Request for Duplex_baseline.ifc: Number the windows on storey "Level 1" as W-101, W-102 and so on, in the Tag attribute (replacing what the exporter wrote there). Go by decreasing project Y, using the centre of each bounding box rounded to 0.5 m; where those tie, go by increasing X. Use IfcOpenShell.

First a look at what the model holds.

```python
import ifcopenshell
import ifcopenshell.util.element
import ifcopenshell.util.placement

model = ifcopenshell.open("Duplex_baseline.ifc")
print(model.schema)
storey = next(s for s in model.by_type("IfcBuildingStorey") if s.Name == "Level 1")
windows = [e for e in ifcopenshell.util.element.get_decomposition(storey) if e.is_a("IfcWindow")]
for e in sorted(windows, key=lambda e: e.id()):
    origin = ifcopenshell.util.placement.get_local_placement(e.ObjectPlacement)[:3, 3]
    print(e.id(), e.Tag, e.Name, origin.round(2) + 0.0, sep=" | ")
```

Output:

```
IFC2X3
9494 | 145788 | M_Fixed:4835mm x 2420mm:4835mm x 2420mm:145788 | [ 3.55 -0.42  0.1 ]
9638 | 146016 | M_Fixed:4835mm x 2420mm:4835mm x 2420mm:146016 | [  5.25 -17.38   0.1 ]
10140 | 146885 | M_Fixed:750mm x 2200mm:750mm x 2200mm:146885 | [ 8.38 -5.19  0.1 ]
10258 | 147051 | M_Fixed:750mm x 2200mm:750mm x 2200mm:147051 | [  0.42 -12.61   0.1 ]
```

```python
import ifcopenshell
import ifcopenshell.geom
import ifcopenshell.util.element
import ifcopenshell.util.shape

model = ifcopenshell.open("Duplex_baseline.ifc")
settings = ifcopenshell.geom.settings()
settings.set("use-world-coords", True)


def centre(element):
    shape = ifcopenshell.geom.create_shape(settings, element)
    return ifcopenshell.util.shape.get_bbox_centroid(shape.geometry)


storey = next(s for s in model.by_type("IfcBuildingStorey") if s.Name == "Level 1")
windows = [e for e in ifcopenshell.util.element.get_decomposition(storey) if e.is_a("IfcWindow")]

# Insertion points can sit at a corner or the storey origin, so sort by the geometry (in metres).
centres = {e: centre(e) for e in windows}
windows.sort(key=lambda e: (-round(centres[e][1] / 0.5), centres[e][0]))

for i, e in enumerate(windows, start=1):
    number = f"W-1{i:02d}"
    e.Tag = number
    print(e.id(), number)

model.write("Duplex_baseline-out.ifc")
```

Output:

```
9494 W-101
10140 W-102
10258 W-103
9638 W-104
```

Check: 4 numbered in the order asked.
